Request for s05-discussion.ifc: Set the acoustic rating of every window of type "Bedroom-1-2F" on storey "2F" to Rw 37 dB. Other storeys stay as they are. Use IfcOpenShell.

First a look at what the model holds.

```python
import ifcopenshell
import ifcopenshell.util.element

model = ifcopenshell.open("s05-discussion.ifc")
print(model.schema)
storey = next(s for s in model.by_type("IfcBuildingStorey") if s.Name == "2F")
windows = [e for e in ifcopenshell.util.element.get_decomposition(storey) if e.is_a("IfcWindow")]
seen = {}
for e in windows:
    element_type = ifcopenshell.util.element.get_type(e)
    key = (element_type.Name if element_type != e and element_type else None, ifcopenshell.util.element.get_pset(e, "Pset_WindowCommon", "AcousticRating"))
    seen[key] = seen.get(key, 0) + 1
for (name, value), count in sorted(seen.items(), key=str):
    print(count, "x", name, "|", value)
```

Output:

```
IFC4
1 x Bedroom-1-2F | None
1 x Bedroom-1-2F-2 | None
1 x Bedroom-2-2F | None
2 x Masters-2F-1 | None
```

```python
import ifcopenshell
import ifcopenshell.api.pset
import ifcopenshell.util.element

model = ifcopenshell.open("s05-discussion.ifc")

storey = next(s for s in model.by_type("IfcBuildingStorey") if s.Name == "2F")
windows = [e for e in ifcopenshell.util.element.get_decomposition(storey) if e.is_a("IfcWindow")]

count = 0
for e in windows:
    element_type = ifcopenshell.util.element.get_type(e)
    if element_type in (None, e) or element_type.Name != "Bedroom-1-2F":
        continue
    # add_pset returns the element's existing set when there is one.
    pset = ifcopenshell.api.pset.add_pset(model, product=e, name="Pset_WindowCommon")
    ifcopenshell.api.pset.edit_pset(model, pset=pset, properties={"AcousticRating": "Rw 37 dB"})
    count += 1

print(count, "windows updated")

model.write("s05-discussion_v2.ifc")
```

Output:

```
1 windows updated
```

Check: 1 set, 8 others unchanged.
